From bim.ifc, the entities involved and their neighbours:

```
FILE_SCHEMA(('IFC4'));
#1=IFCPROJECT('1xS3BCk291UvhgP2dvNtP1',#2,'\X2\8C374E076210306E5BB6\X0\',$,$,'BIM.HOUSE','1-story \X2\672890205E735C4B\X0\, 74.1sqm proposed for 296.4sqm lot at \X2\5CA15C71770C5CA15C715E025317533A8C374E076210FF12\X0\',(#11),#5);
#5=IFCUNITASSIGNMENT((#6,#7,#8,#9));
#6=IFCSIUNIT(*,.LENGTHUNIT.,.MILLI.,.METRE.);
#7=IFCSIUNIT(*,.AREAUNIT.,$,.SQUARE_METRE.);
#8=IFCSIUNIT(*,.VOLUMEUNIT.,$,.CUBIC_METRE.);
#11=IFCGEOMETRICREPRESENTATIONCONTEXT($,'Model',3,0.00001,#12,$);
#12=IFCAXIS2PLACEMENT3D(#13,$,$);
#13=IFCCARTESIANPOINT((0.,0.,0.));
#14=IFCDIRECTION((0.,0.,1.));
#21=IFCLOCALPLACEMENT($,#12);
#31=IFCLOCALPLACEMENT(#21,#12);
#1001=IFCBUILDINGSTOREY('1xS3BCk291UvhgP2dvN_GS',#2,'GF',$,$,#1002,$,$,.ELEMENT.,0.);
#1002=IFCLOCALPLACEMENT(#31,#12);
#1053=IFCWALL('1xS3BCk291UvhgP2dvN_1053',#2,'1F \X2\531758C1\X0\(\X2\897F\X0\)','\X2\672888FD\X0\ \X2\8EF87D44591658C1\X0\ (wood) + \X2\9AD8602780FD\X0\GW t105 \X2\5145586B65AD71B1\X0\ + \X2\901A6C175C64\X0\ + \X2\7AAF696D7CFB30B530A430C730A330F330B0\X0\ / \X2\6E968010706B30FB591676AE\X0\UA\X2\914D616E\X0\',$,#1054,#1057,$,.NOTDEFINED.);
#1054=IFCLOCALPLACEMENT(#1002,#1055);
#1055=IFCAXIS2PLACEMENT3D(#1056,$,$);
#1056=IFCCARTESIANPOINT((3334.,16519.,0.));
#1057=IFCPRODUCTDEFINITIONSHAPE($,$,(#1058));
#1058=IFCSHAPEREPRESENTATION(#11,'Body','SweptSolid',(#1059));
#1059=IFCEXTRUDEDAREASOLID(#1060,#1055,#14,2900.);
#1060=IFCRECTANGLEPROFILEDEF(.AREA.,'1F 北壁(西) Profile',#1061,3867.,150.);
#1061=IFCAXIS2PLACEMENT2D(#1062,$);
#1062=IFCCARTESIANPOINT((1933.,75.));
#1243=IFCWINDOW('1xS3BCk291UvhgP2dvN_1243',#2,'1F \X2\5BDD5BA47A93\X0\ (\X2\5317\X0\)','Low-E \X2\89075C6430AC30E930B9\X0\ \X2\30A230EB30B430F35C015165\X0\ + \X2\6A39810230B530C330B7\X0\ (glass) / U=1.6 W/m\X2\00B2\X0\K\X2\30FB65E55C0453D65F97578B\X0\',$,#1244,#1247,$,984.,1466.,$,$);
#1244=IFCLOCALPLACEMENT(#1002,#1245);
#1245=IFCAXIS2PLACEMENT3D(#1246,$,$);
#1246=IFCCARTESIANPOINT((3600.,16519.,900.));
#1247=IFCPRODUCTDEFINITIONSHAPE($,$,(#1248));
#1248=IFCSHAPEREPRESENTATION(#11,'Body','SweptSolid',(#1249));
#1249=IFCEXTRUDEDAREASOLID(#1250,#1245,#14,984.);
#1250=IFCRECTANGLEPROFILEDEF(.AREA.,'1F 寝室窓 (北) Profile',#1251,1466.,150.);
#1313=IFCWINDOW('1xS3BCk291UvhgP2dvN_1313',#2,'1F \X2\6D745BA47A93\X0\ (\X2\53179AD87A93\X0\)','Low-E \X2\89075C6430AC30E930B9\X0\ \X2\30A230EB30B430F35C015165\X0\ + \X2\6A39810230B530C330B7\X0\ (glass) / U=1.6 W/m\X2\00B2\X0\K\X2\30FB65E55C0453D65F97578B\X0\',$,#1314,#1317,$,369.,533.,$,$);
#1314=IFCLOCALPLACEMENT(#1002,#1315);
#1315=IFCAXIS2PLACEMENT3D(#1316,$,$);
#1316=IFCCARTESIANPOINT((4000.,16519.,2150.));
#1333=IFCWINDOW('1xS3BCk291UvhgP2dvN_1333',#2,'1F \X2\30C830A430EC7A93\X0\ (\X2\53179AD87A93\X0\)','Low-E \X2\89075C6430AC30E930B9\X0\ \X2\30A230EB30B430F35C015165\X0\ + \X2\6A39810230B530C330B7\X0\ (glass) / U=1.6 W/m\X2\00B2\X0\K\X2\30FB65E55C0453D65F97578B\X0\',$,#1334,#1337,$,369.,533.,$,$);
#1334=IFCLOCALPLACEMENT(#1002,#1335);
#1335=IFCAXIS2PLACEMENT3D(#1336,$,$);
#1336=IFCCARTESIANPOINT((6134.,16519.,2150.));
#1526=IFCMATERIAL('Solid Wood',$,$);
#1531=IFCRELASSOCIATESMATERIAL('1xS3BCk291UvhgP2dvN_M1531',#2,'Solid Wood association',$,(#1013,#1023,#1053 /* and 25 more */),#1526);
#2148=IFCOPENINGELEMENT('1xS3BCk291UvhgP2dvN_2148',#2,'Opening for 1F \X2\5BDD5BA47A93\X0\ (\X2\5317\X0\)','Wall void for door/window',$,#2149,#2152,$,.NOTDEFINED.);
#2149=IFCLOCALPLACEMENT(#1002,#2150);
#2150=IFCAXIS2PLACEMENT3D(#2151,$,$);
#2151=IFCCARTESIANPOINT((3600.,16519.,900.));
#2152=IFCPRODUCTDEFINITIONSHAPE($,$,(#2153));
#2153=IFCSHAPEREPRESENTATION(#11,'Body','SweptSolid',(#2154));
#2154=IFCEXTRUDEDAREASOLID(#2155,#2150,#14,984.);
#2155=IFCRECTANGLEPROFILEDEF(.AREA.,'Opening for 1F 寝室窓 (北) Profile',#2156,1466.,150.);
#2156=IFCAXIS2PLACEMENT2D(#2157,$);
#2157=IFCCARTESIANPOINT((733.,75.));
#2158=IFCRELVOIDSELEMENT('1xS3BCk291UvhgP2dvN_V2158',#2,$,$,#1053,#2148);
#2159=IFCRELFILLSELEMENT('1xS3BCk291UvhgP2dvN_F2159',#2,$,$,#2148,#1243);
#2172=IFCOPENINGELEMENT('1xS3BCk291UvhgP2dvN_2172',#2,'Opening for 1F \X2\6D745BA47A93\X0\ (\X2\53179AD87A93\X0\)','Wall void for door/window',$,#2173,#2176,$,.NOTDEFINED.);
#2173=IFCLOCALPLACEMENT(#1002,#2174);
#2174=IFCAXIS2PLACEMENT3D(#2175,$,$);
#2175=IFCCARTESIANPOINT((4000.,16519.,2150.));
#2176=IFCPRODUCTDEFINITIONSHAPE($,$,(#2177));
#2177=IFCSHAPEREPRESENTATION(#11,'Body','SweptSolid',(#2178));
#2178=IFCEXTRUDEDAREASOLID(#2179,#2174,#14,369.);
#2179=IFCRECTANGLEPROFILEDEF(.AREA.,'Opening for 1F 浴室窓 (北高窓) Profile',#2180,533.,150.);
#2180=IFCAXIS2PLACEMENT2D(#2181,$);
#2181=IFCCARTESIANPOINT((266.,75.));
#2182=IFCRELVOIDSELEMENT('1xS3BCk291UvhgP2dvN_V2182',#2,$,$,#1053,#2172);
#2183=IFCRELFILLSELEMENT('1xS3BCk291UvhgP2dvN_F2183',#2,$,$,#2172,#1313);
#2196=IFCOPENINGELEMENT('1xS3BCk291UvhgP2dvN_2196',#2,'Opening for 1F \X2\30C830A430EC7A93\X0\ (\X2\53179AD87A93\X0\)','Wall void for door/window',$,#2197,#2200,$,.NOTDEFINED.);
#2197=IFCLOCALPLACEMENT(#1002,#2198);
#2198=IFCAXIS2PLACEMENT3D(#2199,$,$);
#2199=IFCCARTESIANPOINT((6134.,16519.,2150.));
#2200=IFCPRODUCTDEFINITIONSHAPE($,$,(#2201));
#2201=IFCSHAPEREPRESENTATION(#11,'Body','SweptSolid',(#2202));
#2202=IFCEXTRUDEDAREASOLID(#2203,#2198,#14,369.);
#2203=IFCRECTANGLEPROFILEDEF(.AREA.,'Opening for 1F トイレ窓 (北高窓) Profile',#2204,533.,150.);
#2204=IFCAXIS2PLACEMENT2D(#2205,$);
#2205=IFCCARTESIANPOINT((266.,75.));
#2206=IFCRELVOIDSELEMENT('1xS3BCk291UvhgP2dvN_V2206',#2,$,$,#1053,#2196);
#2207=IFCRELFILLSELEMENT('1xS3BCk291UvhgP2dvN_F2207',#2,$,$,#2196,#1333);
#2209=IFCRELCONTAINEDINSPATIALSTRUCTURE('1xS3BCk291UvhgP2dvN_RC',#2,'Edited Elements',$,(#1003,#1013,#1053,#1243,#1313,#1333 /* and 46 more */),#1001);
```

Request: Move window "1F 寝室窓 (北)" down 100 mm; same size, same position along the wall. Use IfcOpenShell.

```python
import numpy as np
import ifcopenshell
import ifcopenshell.api.geometry
import ifcopenshell.util.placement
import ifcopenshell.util.unit

model = ifcopenshell.open("bim.ifc")
unit_scale = ifcopenshell.util.unit.calculate_unit_scale(model)

window = model.by_guid("1xS3BCk291UvhgP2dvN_1243")
opening = window.FillsVoids[0].RelatingOpeningElement
dz = -0.1 / unit_scale

shift = np.array([0.0, 0.0, dz])
# The window is not placed relative to its opening, so move both.
for product in (opening, window):
    matrix = ifcopenshell.util.placement.get_local_placement(product.ObjectPlacement)
    matrix[:3, 3] += shift
    ifcopenshell.api.geometry.edit_object_placement(model, product=product, matrix=matrix, is_si=False)

print(f"moved by {dz * unit_scale:+.3f} m")

model.write("bim_updated.ifc")
```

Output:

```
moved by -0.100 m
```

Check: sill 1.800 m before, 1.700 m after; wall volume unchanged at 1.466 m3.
